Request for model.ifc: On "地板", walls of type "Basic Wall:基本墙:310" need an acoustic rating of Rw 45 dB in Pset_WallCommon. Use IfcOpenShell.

First a look at what the model holds.

```python
import ifcopenshell
import ifcopenshell.util.element

model = ifcopenshell.open("model.ifc")
print(model.schema)
storey = next(s for s in model.by_type("IfcBuildingStorey") if s.Name == "地板")
walls = [e for e in ifcopenshell.util.element.get_decomposition(storey) if e.is_a("IfcWall")]
seen = {}
for e in walls:
    element_type = ifcopenshell.util.element.get_type(e)
    key = (element_type.Name if element_type != e and element_type else None, ifcopenshell.util.element.get_pset(e, "Pset_WallCommon", "AcousticRating"))
    seen[key] = seen.get(key, 0) + 1
for (name, value), count in sorted(seen.items(), key=str):
    print(count, "x", name, "|", value)
```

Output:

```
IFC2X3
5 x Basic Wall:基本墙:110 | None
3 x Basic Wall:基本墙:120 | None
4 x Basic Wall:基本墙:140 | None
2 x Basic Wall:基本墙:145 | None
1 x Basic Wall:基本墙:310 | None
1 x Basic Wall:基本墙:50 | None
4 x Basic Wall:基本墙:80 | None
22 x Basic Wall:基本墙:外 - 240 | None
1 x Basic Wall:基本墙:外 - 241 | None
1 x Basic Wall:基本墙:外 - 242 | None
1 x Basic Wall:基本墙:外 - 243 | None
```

```python
import ifcopenshell
import ifcopenshell.api.pset
import ifcopenshell.util.element

model = ifcopenshell.open("model.ifc")

storey = next(s for s in model.by_type("IfcBuildingStorey") if s.Name == "地板")
walls = [e for e in ifcopenshell.util.element.get_decomposition(storey) if e.is_a("IfcWall")]

count = 0
for e in walls:
    element_type = ifcopenshell.util.element.get_type(e)
    if element_type in (None, e) or element_type.Name != "Basic Wall:基本墙:310":
        continue
    # add_pset returns the element's existing set when there is one.
    pset = ifcopenshell.api.pset.add_pset(model, product=e, name="Pset_WallCommon")
    ifcopenshell.api.pset.edit_pset(model, pset=pset, properties={"AcousticRating": "Rw 45 dB"})
    count += 1

print(count, "walls updated")

model.write("model_updated.ifc")
```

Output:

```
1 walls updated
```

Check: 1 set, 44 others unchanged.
